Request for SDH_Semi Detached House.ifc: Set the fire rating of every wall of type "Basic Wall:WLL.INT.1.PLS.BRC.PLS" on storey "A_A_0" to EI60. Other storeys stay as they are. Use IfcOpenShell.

First a look at what the model holds.

```python
import ifcopenshell
import ifcopenshell.util.element

model = ifcopenshell.open("SDH_Semi Detached House.ifc")
print(model.schema)
storey = next(s for s in model.by_type("IfcBuildingStorey") if s.Name == "A_A_0")
walls = [e for e in ifcopenshell.util.element.get_decomposition(storey) if e.is_a("IfcWall")]
seen = {}
for e in walls:
    element_type = ifcopenshell.util.element.get_type(e)
    key = (element_type.Name if element_type != e and element_type else None, ifcopenshell.util.element.get_pset(e, "Pset_WallCommon", "FireRating"))
    seen[key] = seen.get(key, 0) + 1
for (name, value), count in sorted(seen.items(), key=str):
    print(count, "x", name, "|", value)
```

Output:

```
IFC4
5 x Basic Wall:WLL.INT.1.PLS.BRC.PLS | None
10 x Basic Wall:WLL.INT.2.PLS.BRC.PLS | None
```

```python
import ifcopenshell
import ifcopenshell.api.pset
import ifcopenshell.util.element

model = ifcopenshell.open("SDH_Semi Detached House.ifc")

storey = next(s for s in model.by_type("IfcBuildingStorey") if s.Name == "A_A_0")
walls = [e for e in ifcopenshell.util.element.get_decomposition(storey) if e.is_a("IfcWall")]

count = 0
for e in walls:
    element_type = ifcopenshell.util.element.get_type(e)
    if element_type in (None, e) or element_type.Name != "Basic Wall:WLL.INT.1.PLS.BRC.PLS":
        continue
    # add_pset returns the element's existing set when there is one.
    pset = ifcopenshell.api.pset.add_pset(model, product=e, name="Pset_WallCommon")
    ifcopenshell.api.pset.edit_pset(model, pset=pset, properties={"FireRating": "EI60"})
    count += 1

print(count, "walls updated")

model.write("SDH_Semi Detached House_rev.ifc")
```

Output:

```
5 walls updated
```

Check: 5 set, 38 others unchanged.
